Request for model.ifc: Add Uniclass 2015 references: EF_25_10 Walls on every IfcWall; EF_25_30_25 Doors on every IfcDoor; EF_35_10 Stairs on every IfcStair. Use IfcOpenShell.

First a look at what the model holds.

```python
import ifcopenshell

model = ifcopenshell.open("model.ifc")
print(model.schema)
print("classifications:", [c.Name for c in model.by_type("IfcClassification")])
for ifc_class in ("IfcDoor", "IfcRoof", "IfcStair", "IfcWall", "IfcWindow"):
    print(ifc_class, len(model.by_type(ifc_class)))
```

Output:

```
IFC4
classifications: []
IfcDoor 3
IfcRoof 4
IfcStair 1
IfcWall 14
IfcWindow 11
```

```python
import ifcopenshell
import ifcopenshell.api.classification

model = ifcopenshell.open("model.ifc")

system = ifcopenshell.api.classification.add_classification(model, classification="Uniclass 2015")

codes = {
    "IfcWall": ("EF_25_10", "Walls"),
    "IfcDoor": ("EF_25_30_25", "Doors"),
    "IfcStair": ("EF_35_10", "Stairs"),
}
for ifc_class, (code, name) in codes.items():
    products = model.by_type(ifc_class)
    ifcopenshell.api.classification.add_reference(
        model, products=products, classification=system, identification=code, name=name
    )
    print(code, len(products))

model.write("model_edited.ifc")
```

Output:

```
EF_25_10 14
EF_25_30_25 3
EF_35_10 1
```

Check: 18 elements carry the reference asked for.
